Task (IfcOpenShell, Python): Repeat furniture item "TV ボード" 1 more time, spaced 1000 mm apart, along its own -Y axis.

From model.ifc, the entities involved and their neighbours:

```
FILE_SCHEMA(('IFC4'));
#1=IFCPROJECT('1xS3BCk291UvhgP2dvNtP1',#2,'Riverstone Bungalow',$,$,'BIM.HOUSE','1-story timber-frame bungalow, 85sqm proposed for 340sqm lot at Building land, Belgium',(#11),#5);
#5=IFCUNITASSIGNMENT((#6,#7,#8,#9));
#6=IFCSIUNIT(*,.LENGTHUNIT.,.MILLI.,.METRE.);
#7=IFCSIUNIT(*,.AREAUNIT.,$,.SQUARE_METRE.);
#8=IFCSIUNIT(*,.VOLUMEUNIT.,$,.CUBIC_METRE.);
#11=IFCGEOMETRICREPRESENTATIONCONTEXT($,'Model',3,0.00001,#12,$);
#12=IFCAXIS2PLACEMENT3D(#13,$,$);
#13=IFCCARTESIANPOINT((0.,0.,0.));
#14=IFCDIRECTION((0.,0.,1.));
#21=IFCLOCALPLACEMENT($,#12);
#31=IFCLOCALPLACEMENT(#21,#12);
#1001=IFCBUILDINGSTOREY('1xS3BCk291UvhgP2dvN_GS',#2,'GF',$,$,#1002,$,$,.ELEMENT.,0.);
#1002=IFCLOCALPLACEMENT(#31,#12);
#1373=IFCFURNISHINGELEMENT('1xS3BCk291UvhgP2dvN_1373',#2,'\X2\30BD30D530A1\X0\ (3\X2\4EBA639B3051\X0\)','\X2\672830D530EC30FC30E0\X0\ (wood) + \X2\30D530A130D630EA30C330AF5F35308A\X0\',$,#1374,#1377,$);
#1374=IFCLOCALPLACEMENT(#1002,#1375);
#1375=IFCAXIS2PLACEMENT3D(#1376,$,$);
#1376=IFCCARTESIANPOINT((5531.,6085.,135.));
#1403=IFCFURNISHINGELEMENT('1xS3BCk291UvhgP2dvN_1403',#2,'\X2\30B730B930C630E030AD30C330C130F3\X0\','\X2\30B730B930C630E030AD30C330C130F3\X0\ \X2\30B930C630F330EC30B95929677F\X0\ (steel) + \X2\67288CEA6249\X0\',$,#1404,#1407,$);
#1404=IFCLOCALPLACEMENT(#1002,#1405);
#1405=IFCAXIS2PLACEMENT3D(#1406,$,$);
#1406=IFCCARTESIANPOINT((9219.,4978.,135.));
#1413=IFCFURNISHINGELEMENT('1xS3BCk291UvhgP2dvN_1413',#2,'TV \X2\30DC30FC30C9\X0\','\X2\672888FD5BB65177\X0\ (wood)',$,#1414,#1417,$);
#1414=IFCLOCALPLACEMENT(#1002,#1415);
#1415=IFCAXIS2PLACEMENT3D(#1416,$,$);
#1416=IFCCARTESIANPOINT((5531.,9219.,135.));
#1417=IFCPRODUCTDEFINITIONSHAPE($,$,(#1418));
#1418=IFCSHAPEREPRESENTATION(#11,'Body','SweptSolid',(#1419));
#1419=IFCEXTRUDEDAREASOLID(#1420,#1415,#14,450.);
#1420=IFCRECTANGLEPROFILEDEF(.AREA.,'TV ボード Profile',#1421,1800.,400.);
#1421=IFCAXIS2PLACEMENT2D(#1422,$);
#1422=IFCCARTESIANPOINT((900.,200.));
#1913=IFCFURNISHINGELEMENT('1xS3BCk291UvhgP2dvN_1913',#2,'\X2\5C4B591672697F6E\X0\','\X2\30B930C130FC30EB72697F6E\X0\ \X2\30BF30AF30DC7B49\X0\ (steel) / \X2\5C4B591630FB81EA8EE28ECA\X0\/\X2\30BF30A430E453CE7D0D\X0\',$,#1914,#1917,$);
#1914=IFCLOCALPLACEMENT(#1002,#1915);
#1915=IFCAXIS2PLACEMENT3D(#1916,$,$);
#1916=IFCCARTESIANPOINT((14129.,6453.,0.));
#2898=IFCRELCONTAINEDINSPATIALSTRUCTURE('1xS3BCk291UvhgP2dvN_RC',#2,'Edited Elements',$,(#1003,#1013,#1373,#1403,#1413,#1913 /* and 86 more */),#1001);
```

```python
import ifcopenshell
import ifcopenshell.api.geometry
import ifcopenshell.api.root
import ifcopenshell.util.element
import ifcopenshell.util.placement

model = ifcopenshell.open("model.ifc")


def reuse_history(source, copy):
    """copy_class also copies each property set's owner history, people and application; keep the originals."""
    for rel in copy.IsDefinedBy:
        if rel.is_a("IfcRelDefinesByProperties") and (history := rel.RelatingPropertyDefinition.OwnerHistory):
            rel.RelatingPropertyDefinition.OwnerHistory = source.OwnerHistory
            ifcopenshell.util.element.remove_deep2(model, history)


source = model.by_id(1413)
base = ifcopenshell.util.placement.get_local_placement(source.ObjectPlacement)
step = -base[:3, 1] * 1000.0

for i in range(1, 2):
    copy = ifcopenshell.api.root.copy_class(model, product=source)
    copy.Representation = ifcopenshell.util.element.copy_deep(
        model, source.Representation, exclude=["IfcGeometricRepresentationContext", "IfcRepresentationMap"]
    )
    reuse_history(source, copy)
    matrix = base.copy()
    matrix[:3, 3] += i * step
    print("added at", matrix[:3, 3].round(3) + 0.0)
    ifcopenshell.api.geometry.edit_object_placement(model, product=copy, matrix=matrix, is_si=False)

model.write("model_updated.ifc")
```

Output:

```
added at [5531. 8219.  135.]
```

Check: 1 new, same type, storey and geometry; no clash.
